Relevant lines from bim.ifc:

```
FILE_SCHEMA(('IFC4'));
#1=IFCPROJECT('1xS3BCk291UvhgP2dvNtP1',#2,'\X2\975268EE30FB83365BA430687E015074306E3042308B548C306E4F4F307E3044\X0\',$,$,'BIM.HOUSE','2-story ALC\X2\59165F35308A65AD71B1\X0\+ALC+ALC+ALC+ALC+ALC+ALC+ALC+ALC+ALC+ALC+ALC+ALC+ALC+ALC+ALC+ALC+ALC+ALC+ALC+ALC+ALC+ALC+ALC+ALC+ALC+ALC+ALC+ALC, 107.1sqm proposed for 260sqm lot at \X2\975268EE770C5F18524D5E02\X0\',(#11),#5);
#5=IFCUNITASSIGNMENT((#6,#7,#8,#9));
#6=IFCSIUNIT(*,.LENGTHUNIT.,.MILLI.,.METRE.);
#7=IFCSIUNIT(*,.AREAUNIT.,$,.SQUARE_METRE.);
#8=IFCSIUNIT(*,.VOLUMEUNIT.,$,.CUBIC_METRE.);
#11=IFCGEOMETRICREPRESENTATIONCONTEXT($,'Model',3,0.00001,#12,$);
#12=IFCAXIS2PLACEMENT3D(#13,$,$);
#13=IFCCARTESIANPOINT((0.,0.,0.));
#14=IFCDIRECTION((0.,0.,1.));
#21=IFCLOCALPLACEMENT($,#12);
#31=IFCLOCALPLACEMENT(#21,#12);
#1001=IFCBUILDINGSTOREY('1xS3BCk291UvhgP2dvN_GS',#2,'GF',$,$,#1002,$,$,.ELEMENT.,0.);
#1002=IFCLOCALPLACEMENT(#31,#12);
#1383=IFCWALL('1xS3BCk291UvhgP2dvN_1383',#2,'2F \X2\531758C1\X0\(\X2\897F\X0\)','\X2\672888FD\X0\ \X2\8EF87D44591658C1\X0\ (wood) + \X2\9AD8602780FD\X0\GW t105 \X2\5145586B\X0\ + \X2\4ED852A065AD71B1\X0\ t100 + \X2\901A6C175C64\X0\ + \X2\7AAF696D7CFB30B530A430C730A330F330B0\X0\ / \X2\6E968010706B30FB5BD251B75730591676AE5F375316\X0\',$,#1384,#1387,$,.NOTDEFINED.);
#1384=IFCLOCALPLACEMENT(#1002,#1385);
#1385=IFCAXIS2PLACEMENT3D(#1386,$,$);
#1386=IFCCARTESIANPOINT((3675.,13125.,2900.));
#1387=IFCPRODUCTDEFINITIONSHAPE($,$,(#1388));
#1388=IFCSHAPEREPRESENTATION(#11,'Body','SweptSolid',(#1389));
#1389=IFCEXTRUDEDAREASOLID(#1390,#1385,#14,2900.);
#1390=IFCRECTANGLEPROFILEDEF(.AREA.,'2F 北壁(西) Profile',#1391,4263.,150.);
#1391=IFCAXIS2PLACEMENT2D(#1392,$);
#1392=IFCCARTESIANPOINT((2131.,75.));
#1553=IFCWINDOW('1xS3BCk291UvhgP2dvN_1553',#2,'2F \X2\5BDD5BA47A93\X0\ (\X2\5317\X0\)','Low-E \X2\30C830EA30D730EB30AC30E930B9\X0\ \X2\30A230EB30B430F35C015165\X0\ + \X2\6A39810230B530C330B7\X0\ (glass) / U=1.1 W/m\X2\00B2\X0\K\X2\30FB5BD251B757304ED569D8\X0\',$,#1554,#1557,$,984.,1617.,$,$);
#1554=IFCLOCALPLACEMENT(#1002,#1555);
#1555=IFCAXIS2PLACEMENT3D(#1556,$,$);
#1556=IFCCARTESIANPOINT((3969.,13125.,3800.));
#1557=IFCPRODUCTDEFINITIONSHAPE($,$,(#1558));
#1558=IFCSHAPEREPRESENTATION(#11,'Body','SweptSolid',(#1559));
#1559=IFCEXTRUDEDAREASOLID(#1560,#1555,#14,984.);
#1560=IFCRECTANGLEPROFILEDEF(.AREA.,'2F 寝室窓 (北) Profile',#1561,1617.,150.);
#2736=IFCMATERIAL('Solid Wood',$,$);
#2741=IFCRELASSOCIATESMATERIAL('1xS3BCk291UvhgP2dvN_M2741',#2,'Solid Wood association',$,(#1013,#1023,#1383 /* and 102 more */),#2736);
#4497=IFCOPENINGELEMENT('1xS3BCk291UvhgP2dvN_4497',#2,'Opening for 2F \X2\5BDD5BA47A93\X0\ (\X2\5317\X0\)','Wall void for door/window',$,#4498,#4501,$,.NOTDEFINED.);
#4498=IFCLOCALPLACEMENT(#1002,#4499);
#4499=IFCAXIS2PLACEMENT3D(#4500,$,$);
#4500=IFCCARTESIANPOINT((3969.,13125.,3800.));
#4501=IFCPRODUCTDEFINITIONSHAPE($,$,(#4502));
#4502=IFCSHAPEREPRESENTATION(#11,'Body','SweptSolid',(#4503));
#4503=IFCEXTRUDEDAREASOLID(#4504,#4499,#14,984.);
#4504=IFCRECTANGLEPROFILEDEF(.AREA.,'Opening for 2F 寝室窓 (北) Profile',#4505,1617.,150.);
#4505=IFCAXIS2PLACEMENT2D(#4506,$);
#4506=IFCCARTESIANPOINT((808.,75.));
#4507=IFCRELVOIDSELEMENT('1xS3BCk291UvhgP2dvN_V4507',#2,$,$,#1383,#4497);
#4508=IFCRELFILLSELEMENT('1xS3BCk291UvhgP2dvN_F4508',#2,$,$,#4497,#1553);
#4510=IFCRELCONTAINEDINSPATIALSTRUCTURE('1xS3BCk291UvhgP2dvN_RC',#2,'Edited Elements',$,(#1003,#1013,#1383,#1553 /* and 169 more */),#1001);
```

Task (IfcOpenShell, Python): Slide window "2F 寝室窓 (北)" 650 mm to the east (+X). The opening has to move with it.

```python
import ifcopenshell
import ifcopenshell.api.geometry
import ifcopenshell.util.placement
import ifcopenshell.util.unit

model = ifcopenshell.open("bim.ifc")
unit_scale = ifcopenshell.util.unit.calculate_unit_scale(model)

window = model.by_id(1553)
opening = window.FillsVoids[0].RelatingOpeningElement
wall = opening.VoidsElements[0].RelatingBuildingElement

wall_matrix = ifcopenshell.util.placement.get_local_placement(wall.ObjectPlacement)
shift = wall_matrix[:3, 0] * 0.65 / unit_scale
before = ifcopenshell.util.placement.get_local_placement(window.ObjectPlacement)[:3, 3].copy()

# The window is not placed relative to its opening, so move both.
for product in (opening, window):
    matrix = ifcopenshell.util.placement.get_local_placement(product.ObjectPlacement)
    matrix[:3, 3] += shift
    ifcopenshell.api.geometry.edit_object_placement(model, product=product, matrix=matrix, is_si=False)

after = ifcopenshell.util.placement.get_local_placement(window.ObjectPlacement)[:3, 3]
print("window moved by", (after - before).round(3) + 0.0)

model.write("bim_rev.ifc")
```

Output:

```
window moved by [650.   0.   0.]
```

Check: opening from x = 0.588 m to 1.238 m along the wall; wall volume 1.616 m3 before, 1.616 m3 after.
